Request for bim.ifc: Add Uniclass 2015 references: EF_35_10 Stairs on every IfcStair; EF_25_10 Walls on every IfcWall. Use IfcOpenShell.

First a look at what the model holds.

```python
import ifcopenshell

model = ifcopenshell.open("bim.ifc")
print(model.schema)
print("classifications:", [c.Name for c in model.by_type("IfcClassification")])
for ifc_class in ("IfcDoor", "IfcRoof", "IfcStair", "IfcWall", "IfcWindow"):
    print(ifc_class, len(model.by_type(ifc_class)))
```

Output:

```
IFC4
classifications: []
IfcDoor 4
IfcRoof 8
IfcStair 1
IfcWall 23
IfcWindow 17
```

```python
import ifcopenshell
import ifcopenshell.api.classification

model = ifcopenshell.open("bim.ifc")

system = ifcopenshell.api.classification.add_classification(model, classification="Uniclass 2015")

codes = {
    "IfcStair": ("EF_35_10", "Stairs"),
    "IfcWall": ("EF_25_10", "Walls"),
}
for ifc_class, (code, name) in codes.items():
    products = model.by_type(ifc_class)
    ifcopenshell.api.classification.add_reference(
        model, products=products, classification=system, identification=code, name=name
    )
    print(code, len(products))

model.write("bim_updated.ifc")
```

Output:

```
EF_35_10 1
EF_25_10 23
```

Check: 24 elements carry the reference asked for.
